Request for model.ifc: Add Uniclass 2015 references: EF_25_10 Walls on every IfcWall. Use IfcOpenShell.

First a look at what the model holds.

```python
import ifcopenshell

model = ifcopenshell.open("model.ifc")
print(model.schema)
print("classifications:", [c.Name for c in model.by_type("IfcClassification")])
for ifc_class in ("IfcDoor", "IfcRoof", "IfcStair", "IfcWall", "IfcWindow"):
    print(ifc_class, len(model.by_type(ifc_class)))
```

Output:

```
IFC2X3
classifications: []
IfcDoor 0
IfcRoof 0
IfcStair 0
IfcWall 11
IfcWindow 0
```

```python
import ifcopenshell
import ifcopenshell.api.classification

model = ifcopenshell.open("model.ifc")

# IFC2X3 requires Source and Edition and has no link from the project to the system.
system = model.create_entity("IfcClassification", Source="NBS", Edition="2015", Name="Uniclass 2015")

codes = {
    "IfcWall": ("EF_25_10", "Walls"),
}
for ifc_class, (code, name) in codes.items():
    products = model.by_type(ifc_class)
    ifcopenshell.api.classification.add_reference(
        model, products=products, classification=system, identification=code, name=name
    )
    print(code, len(products))

model.write("model_v2.ifc")
```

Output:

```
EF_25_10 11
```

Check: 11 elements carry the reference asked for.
